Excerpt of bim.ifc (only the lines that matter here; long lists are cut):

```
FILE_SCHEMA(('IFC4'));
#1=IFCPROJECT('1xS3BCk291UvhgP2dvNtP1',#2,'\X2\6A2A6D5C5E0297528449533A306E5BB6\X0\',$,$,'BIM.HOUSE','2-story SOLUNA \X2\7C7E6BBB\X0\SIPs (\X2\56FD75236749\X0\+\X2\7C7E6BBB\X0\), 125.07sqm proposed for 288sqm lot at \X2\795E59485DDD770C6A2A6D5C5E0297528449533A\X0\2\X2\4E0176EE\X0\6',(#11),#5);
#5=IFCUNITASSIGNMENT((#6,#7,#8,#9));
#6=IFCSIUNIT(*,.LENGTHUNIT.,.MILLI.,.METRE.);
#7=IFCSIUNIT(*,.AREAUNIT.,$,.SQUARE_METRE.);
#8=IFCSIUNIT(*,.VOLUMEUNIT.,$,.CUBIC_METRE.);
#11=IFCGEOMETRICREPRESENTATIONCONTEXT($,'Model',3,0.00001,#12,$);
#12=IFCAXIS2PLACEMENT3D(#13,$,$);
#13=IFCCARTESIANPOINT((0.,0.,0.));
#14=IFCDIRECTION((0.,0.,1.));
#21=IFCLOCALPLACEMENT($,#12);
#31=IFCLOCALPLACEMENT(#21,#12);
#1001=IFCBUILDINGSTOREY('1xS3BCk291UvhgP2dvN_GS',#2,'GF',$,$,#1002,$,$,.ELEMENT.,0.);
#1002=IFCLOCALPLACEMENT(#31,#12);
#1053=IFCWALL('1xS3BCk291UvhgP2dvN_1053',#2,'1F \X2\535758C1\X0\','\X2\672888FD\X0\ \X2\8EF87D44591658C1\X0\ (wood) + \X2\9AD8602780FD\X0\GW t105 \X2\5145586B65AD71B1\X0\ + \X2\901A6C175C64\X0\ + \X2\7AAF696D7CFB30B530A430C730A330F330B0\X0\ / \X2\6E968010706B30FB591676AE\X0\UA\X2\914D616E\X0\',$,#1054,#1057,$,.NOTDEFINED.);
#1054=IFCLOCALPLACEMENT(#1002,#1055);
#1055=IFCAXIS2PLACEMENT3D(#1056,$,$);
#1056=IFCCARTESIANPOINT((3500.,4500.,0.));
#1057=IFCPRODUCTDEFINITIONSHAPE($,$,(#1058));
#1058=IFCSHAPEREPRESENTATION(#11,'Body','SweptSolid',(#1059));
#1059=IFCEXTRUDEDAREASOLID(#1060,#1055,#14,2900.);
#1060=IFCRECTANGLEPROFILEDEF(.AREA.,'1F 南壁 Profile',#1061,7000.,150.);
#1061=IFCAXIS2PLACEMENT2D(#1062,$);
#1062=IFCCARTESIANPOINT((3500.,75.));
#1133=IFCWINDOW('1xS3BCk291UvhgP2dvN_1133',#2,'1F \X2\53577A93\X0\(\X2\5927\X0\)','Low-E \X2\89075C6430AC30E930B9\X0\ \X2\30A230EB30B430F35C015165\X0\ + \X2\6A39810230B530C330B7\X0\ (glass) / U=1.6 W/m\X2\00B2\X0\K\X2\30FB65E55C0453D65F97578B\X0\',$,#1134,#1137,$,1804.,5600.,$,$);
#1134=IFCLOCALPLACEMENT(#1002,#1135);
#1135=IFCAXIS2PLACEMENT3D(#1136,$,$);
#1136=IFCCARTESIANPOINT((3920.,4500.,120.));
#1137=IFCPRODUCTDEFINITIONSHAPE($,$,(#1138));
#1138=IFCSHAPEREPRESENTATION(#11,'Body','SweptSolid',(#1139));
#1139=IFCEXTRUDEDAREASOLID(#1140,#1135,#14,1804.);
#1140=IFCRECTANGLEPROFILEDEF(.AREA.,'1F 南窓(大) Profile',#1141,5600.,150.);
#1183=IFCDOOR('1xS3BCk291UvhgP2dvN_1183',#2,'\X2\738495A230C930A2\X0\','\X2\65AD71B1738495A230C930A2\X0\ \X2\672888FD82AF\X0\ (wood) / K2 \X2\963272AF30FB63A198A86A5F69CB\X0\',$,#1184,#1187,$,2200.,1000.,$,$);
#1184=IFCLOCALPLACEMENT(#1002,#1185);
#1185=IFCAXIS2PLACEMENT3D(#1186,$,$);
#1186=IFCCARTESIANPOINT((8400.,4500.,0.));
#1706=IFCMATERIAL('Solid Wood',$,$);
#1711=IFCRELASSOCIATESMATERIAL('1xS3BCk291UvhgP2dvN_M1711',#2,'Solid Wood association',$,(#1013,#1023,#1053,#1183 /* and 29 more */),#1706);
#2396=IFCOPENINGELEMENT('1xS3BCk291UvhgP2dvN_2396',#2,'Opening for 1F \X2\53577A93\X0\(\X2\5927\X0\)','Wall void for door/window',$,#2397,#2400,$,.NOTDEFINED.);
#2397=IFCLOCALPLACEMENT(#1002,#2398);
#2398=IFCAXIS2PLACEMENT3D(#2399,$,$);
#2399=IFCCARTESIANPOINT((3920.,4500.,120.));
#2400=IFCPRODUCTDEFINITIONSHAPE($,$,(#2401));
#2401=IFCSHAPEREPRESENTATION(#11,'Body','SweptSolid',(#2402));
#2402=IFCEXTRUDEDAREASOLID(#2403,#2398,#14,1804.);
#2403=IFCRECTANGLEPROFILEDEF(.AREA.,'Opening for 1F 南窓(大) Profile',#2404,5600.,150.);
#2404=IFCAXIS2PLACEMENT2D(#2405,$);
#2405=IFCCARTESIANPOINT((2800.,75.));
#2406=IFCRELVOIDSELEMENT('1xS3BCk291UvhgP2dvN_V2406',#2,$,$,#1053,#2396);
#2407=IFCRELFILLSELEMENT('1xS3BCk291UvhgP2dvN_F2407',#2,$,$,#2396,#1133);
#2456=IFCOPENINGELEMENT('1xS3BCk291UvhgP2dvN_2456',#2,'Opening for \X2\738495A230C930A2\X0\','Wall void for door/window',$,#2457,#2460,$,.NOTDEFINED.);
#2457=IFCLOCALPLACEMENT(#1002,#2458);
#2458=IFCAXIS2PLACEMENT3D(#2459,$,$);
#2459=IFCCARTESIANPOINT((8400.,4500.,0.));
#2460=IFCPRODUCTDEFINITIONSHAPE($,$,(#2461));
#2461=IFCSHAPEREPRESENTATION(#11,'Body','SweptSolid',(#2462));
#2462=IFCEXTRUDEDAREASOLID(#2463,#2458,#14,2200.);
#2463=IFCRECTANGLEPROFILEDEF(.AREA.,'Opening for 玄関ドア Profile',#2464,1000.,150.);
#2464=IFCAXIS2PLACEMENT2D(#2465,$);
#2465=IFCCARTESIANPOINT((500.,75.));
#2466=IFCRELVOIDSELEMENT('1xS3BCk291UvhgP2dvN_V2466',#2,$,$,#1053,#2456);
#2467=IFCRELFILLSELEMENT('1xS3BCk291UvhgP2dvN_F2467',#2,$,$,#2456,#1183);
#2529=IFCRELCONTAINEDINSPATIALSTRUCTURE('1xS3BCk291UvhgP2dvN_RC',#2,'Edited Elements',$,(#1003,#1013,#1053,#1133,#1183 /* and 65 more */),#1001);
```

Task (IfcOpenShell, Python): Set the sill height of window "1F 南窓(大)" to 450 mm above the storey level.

```python
import numpy as np
import ifcopenshell
import ifcopenshell.api.geometry
import ifcopenshell.geom
import ifcopenshell.util.element
import ifcopenshell.util.placement
import ifcopenshell.util.shape
import ifcopenshell.util.unit

model = ifcopenshell.open("bim.ifc")
unit_scale = ifcopenshell.util.unit.calculate_unit_scale(model)

window = model.by_guid("1xS3BCk291UvhgP2dvN_1133")
opening = window.FillsVoids[0].RelatingOpeningElement
storey = ifcopenshell.util.element.get_container(window, ifc_class="IfcBuildingStorey")
level = ifcopenshell.util.placement.get_local_placement(storey.ObjectPlacement)[2, 3]

# The opening's origin need not be at the sill, so measure its lowest point.
shape = ifcopenshell.geom.create_shape(ifcopenshell.geom.settings(), opening)
bottom = ifcopenshell.util.shape.get_shape_bottom_elevation(shape, shape.geometry) / unit_scale
dz = level + 0.45 / unit_scale - bottom

shift = np.array([0.0, 0.0, dz])
# The window is not placed relative to its opening, so move both.
for product in (opening, window):
    matrix = ifcopenshell.util.placement.get_local_placement(product.ObjectPlacement)
    matrix[:3, 3] += shift
    ifcopenshell.api.geometry.edit_object_placement(model, product=product, matrix=matrix, is_si=False)

print(f"moved by {dz * unit_scale:+.3f} m")

model.write("bim-out.ifc")
```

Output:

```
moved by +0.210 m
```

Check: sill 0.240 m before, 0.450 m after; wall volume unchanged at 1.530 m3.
